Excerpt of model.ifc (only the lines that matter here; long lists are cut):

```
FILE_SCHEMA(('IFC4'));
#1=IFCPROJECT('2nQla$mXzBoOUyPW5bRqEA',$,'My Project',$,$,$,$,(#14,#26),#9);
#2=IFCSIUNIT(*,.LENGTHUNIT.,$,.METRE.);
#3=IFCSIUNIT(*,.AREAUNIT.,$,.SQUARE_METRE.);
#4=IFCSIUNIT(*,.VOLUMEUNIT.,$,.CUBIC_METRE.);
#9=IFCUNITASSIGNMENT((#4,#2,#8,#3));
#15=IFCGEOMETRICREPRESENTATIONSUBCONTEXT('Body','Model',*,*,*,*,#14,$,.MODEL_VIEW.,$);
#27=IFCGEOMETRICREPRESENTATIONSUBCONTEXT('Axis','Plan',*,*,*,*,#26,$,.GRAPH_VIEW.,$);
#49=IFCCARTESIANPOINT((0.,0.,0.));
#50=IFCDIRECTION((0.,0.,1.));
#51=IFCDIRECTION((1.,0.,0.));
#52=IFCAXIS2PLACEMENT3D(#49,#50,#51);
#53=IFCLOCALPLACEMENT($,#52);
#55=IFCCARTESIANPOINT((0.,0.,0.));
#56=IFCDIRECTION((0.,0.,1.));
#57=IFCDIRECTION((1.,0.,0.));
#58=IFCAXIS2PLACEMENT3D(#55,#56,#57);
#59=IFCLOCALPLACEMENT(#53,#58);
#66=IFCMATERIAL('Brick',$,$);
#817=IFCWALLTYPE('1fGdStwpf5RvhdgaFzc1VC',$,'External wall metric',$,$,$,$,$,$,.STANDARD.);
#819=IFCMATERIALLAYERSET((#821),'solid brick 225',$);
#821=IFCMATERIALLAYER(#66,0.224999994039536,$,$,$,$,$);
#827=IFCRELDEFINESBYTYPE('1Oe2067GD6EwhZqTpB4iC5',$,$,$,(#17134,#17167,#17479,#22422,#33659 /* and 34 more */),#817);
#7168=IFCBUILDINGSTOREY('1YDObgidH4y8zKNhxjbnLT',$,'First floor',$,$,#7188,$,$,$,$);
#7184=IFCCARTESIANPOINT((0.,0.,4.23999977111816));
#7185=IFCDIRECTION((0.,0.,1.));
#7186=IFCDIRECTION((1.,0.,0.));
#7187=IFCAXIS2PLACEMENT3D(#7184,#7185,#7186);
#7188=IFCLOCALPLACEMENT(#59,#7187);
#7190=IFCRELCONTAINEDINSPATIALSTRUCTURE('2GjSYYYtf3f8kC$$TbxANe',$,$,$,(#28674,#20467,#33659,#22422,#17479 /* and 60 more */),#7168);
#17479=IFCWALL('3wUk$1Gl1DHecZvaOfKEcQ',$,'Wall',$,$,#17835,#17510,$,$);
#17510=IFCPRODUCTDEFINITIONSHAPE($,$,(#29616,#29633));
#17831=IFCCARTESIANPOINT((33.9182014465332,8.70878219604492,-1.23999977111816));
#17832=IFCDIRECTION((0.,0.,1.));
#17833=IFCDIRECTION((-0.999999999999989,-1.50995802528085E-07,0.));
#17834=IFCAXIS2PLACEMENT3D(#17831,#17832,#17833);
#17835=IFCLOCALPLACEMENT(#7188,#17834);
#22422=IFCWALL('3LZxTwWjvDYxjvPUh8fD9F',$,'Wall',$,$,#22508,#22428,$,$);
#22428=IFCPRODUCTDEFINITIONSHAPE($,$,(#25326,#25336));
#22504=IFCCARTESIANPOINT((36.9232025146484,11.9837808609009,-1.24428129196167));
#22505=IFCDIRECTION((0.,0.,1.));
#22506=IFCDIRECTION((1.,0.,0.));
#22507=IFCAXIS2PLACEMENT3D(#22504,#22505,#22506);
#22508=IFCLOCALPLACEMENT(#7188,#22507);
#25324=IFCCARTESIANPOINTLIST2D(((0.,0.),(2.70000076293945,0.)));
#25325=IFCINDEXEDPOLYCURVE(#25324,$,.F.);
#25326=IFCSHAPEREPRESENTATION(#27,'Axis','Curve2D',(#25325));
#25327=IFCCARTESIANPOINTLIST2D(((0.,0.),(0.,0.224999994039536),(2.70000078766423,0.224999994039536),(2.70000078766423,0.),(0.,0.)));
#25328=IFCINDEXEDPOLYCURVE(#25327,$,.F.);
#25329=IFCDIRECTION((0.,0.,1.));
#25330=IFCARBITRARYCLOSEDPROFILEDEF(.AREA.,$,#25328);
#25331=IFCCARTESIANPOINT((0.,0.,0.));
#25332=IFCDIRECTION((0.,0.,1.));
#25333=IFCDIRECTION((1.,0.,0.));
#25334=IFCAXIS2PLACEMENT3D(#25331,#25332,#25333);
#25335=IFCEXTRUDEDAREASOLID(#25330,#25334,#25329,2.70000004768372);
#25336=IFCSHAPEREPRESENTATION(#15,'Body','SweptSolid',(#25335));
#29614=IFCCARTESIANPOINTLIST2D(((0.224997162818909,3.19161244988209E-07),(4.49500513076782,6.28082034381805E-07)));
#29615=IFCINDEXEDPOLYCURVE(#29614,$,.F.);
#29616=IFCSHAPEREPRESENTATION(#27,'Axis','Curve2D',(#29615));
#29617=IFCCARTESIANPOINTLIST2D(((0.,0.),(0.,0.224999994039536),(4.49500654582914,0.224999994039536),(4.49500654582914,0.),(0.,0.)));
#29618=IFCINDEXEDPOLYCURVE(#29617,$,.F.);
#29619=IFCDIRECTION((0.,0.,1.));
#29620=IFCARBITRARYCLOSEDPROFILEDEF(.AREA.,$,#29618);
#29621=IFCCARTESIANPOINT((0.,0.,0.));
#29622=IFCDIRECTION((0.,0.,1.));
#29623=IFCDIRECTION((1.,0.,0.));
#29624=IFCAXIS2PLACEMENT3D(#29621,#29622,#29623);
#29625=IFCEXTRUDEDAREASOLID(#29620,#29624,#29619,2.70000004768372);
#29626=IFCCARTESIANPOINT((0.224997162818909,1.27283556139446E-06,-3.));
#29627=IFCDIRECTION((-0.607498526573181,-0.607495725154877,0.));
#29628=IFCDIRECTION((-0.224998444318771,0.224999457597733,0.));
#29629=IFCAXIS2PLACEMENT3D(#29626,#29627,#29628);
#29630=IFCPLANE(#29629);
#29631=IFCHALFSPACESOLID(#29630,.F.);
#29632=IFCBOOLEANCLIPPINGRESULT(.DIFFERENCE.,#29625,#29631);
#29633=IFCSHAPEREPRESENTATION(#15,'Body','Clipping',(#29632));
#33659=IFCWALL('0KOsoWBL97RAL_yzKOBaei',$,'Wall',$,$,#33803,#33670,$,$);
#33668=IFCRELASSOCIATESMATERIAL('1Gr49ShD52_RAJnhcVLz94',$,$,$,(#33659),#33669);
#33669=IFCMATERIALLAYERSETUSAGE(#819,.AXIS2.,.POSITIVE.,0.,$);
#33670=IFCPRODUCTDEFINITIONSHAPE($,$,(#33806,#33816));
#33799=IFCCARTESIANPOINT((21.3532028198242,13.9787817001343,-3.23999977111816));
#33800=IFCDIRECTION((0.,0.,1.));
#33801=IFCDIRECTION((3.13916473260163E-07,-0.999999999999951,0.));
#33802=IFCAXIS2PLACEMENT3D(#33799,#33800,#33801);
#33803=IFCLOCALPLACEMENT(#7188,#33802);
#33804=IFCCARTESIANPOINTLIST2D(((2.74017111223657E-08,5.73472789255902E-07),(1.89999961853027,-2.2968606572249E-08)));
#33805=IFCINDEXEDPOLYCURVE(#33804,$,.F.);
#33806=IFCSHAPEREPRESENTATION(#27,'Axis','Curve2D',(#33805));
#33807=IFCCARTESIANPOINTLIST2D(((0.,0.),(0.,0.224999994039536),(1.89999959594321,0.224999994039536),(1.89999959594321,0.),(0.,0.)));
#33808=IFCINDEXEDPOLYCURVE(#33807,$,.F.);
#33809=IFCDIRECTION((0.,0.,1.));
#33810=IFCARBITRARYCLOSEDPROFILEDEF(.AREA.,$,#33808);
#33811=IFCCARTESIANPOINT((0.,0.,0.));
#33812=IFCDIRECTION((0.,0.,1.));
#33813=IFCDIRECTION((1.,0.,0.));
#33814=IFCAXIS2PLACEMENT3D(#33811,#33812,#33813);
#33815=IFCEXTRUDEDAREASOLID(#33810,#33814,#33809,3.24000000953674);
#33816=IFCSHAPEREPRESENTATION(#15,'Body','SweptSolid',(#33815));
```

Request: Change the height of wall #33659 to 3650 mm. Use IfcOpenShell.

```python
import ifcopenshell
import ifcopenshell.geom
import ifcopenshell.util.representation
import ifcopenshell.util.shape
import ifcopenshell.util.unit

model = ifcopenshell.open("model.ifc")
unit_scale = ifcopenshell.util.unit.calculate_unit_scale(model)
settings = ifcopenshell.geom.settings()


def volume(element):
    """Net volume in cubic metres, openings subtracted."""
    shape = ifcopenshell.geom.create_shape(settings, element)
    return ifcopenshell.util.shape.get_volume(shape.geometry)


wall = model.by_id(33659)
before = volume(wall)

body = ifcopenshell.util.representation.get_representation(wall, "Model", "Body")
solid = body.Items[0]
old_height = solid.Depth
solid.Depth = 3.65 / unit_scale
after = volume(wall)

print(f"height {old_height:g} -> {solid.Depth:g}, volume {before:.3f} -> {after:.3f} m3")

model.write("model_v2.ifc")
```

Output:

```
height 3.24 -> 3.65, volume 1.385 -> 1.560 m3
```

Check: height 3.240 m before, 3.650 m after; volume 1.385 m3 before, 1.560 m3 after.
